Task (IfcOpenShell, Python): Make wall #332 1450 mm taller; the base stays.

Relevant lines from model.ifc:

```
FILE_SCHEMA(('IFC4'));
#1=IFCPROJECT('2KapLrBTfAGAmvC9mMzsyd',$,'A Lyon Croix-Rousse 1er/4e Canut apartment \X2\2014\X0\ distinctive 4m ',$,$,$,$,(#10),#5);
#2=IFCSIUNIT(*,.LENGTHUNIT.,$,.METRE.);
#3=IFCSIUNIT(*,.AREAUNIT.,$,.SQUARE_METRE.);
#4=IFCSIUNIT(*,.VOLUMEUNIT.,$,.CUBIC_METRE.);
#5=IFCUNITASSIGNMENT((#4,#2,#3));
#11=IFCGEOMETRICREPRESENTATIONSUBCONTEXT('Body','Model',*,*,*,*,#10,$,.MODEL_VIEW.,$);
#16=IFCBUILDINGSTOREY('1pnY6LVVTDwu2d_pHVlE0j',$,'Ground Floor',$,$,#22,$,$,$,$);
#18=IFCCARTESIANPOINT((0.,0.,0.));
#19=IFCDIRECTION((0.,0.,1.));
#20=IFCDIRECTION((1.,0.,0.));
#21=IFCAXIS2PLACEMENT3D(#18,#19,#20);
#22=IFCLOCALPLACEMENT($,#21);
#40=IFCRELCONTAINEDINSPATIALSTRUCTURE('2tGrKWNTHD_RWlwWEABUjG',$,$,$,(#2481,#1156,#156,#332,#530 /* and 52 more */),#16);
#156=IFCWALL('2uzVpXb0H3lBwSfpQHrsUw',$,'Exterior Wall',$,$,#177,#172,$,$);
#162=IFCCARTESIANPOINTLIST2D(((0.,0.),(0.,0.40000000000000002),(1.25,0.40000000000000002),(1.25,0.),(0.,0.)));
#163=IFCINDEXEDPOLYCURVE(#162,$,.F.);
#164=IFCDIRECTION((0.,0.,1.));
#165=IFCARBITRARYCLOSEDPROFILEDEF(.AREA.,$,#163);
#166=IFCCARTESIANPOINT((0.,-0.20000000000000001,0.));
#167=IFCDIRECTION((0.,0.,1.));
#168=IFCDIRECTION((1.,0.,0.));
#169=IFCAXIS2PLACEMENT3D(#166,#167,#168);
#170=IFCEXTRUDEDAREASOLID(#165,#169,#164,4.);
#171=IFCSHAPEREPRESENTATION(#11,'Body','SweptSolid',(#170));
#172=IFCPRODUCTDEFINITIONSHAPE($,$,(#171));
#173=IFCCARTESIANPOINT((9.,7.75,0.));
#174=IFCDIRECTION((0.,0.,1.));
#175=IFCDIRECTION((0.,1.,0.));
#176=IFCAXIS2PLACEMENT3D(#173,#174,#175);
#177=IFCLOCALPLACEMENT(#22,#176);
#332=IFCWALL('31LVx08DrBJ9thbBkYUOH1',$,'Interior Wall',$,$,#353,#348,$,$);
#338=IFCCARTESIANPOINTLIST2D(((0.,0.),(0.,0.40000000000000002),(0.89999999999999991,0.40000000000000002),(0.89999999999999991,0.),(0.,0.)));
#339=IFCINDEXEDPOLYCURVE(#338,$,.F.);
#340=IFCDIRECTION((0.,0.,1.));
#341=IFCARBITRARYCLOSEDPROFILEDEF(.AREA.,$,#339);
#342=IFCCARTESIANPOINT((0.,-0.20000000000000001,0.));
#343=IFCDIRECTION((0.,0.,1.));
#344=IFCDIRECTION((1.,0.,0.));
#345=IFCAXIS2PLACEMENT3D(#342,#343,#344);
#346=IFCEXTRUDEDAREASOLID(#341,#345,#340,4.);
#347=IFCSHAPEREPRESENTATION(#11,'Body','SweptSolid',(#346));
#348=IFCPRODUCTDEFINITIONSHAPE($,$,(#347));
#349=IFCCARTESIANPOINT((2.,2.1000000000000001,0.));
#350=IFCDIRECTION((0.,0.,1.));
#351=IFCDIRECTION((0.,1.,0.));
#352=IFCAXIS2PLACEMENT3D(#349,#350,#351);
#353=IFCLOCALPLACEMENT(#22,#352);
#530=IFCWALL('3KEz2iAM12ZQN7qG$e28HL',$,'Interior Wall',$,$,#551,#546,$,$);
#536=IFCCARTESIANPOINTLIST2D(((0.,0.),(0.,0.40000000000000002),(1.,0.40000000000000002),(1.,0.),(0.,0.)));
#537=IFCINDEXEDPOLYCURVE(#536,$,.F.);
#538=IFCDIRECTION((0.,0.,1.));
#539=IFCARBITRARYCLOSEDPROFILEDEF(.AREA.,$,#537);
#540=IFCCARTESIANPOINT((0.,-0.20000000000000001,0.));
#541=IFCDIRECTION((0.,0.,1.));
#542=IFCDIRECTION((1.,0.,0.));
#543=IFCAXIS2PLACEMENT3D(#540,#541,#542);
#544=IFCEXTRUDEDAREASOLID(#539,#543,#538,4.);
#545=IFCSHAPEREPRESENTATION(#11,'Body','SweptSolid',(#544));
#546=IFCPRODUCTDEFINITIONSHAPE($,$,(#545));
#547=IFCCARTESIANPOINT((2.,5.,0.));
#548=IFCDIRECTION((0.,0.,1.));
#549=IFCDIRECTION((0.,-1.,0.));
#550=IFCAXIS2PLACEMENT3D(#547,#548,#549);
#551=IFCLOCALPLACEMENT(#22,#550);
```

```python
import ifcopenshell
import ifcopenshell.geom
import ifcopenshell.util.representation
import ifcopenshell.util.shape

model = ifcopenshell.open("model.ifc")
settings = ifcopenshell.geom.settings()


def volume(element):
    """Net volume in cubic metres, openings subtracted."""
    shape = ifcopenshell.geom.create_shape(settings, element)
    return ifcopenshell.util.shape.get_volume(shape.geometry)


wall = model.by_guid("31LVx08DrBJ9thbBkYUOH1")
before = volume(wall)

body = ifcopenshell.util.representation.get_representation(wall, "Model", "Body")
solid = body.Items[0]
old_height = solid.Depth
solid.Depth += 1.45
after = volume(wall)

print(f"height {old_height:g} -> {solid.Depth:g}, volume {before:.3f} -> {after:.3f} m3")

model.write("model_v2.ifc")
```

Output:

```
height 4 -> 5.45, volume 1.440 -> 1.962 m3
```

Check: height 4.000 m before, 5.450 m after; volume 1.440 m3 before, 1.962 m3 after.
